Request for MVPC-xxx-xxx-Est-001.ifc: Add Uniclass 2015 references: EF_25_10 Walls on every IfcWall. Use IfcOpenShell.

First a look at what the model holds.

```python
import ifcopenshell

model = ifcopenshell.open("MVPC-xxx-xxx-Est-001.ifc")
print(model.schema)
print("classifications:", [c.Name for c in model.by_type("IfcClassification")])
for ifc_class in ("IfcDoor", "IfcRoof", "IfcStair", "IfcWall", "IfcWindow"):
    print(ifc_class, len(model.by_type(ifc_class)))
```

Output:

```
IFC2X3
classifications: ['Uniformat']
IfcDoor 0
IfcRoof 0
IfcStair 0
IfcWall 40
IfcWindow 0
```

```python
import ifcopenshell
import ifcopenshell.api.classification

model = ifcopenshell.open("MVPC-xxx-xxx-Est-001.ifc")

# IFC2X3 requires Source and Edition and has no link from the project to the system.
system = model.create_entity("IfcClassification", Source="NBS", Edition="2015", Name="Uniclass 2015")

codes = {
    "IfcWall": ("EF_25_10", "Walls"),
}
for ifc_class, (code, name) in codes.items():
    products = model.by_type(ifc_class)
    ifcopenshell.api.classification.add_reference(
        model, products=products, classification=system, identification=code, name=name
    )
    print(code, len(products))

model.write("MVPC-xxx-xxx-Est-001_v2.ifc")
```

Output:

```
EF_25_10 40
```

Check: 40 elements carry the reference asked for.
